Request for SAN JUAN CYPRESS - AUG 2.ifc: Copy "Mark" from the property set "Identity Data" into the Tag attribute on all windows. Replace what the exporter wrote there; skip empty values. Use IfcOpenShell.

First a look at what the model holds.

```python
import ifcopenshell
import ifcopenshell.util.element

model = ifcopenshell.open("SAN JUAN CYPRESS - AUG 2.ifc")
print(model.schema)
windows = model.by_type("IfcWindow")
print(len(windows), "windows")
for e in windows[:8]:
    source = ifcopenshell.util.element.get_pset(e, "Identity Data", "Mark")
    target = e.Tag
    print(e.id(), repr(source), repr(target), sep=" | ")
```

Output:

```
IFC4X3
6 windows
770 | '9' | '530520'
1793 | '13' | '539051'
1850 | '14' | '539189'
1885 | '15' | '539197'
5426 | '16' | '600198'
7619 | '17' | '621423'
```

```python
import ifcopenshell
import ifcopenshell.util.element

model = ifcopenshell.open("SAN JUAN CYPRESS - AUG 2.ifc")

count = 0
for e in model.by_type("IfcWindow"):
    value = ifcopenshell.util.element.get_pset(e, "Identity Data", "Mark")
    current = e.Tag
    if not value or not value.strip() or current == value:
        continue
    e.Tag = value
    count += 1

print(count, "windows updated")

model.write("SAN JUAN CYPRESS - AUG 2_updated.ifc")
```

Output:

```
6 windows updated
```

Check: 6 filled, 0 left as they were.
